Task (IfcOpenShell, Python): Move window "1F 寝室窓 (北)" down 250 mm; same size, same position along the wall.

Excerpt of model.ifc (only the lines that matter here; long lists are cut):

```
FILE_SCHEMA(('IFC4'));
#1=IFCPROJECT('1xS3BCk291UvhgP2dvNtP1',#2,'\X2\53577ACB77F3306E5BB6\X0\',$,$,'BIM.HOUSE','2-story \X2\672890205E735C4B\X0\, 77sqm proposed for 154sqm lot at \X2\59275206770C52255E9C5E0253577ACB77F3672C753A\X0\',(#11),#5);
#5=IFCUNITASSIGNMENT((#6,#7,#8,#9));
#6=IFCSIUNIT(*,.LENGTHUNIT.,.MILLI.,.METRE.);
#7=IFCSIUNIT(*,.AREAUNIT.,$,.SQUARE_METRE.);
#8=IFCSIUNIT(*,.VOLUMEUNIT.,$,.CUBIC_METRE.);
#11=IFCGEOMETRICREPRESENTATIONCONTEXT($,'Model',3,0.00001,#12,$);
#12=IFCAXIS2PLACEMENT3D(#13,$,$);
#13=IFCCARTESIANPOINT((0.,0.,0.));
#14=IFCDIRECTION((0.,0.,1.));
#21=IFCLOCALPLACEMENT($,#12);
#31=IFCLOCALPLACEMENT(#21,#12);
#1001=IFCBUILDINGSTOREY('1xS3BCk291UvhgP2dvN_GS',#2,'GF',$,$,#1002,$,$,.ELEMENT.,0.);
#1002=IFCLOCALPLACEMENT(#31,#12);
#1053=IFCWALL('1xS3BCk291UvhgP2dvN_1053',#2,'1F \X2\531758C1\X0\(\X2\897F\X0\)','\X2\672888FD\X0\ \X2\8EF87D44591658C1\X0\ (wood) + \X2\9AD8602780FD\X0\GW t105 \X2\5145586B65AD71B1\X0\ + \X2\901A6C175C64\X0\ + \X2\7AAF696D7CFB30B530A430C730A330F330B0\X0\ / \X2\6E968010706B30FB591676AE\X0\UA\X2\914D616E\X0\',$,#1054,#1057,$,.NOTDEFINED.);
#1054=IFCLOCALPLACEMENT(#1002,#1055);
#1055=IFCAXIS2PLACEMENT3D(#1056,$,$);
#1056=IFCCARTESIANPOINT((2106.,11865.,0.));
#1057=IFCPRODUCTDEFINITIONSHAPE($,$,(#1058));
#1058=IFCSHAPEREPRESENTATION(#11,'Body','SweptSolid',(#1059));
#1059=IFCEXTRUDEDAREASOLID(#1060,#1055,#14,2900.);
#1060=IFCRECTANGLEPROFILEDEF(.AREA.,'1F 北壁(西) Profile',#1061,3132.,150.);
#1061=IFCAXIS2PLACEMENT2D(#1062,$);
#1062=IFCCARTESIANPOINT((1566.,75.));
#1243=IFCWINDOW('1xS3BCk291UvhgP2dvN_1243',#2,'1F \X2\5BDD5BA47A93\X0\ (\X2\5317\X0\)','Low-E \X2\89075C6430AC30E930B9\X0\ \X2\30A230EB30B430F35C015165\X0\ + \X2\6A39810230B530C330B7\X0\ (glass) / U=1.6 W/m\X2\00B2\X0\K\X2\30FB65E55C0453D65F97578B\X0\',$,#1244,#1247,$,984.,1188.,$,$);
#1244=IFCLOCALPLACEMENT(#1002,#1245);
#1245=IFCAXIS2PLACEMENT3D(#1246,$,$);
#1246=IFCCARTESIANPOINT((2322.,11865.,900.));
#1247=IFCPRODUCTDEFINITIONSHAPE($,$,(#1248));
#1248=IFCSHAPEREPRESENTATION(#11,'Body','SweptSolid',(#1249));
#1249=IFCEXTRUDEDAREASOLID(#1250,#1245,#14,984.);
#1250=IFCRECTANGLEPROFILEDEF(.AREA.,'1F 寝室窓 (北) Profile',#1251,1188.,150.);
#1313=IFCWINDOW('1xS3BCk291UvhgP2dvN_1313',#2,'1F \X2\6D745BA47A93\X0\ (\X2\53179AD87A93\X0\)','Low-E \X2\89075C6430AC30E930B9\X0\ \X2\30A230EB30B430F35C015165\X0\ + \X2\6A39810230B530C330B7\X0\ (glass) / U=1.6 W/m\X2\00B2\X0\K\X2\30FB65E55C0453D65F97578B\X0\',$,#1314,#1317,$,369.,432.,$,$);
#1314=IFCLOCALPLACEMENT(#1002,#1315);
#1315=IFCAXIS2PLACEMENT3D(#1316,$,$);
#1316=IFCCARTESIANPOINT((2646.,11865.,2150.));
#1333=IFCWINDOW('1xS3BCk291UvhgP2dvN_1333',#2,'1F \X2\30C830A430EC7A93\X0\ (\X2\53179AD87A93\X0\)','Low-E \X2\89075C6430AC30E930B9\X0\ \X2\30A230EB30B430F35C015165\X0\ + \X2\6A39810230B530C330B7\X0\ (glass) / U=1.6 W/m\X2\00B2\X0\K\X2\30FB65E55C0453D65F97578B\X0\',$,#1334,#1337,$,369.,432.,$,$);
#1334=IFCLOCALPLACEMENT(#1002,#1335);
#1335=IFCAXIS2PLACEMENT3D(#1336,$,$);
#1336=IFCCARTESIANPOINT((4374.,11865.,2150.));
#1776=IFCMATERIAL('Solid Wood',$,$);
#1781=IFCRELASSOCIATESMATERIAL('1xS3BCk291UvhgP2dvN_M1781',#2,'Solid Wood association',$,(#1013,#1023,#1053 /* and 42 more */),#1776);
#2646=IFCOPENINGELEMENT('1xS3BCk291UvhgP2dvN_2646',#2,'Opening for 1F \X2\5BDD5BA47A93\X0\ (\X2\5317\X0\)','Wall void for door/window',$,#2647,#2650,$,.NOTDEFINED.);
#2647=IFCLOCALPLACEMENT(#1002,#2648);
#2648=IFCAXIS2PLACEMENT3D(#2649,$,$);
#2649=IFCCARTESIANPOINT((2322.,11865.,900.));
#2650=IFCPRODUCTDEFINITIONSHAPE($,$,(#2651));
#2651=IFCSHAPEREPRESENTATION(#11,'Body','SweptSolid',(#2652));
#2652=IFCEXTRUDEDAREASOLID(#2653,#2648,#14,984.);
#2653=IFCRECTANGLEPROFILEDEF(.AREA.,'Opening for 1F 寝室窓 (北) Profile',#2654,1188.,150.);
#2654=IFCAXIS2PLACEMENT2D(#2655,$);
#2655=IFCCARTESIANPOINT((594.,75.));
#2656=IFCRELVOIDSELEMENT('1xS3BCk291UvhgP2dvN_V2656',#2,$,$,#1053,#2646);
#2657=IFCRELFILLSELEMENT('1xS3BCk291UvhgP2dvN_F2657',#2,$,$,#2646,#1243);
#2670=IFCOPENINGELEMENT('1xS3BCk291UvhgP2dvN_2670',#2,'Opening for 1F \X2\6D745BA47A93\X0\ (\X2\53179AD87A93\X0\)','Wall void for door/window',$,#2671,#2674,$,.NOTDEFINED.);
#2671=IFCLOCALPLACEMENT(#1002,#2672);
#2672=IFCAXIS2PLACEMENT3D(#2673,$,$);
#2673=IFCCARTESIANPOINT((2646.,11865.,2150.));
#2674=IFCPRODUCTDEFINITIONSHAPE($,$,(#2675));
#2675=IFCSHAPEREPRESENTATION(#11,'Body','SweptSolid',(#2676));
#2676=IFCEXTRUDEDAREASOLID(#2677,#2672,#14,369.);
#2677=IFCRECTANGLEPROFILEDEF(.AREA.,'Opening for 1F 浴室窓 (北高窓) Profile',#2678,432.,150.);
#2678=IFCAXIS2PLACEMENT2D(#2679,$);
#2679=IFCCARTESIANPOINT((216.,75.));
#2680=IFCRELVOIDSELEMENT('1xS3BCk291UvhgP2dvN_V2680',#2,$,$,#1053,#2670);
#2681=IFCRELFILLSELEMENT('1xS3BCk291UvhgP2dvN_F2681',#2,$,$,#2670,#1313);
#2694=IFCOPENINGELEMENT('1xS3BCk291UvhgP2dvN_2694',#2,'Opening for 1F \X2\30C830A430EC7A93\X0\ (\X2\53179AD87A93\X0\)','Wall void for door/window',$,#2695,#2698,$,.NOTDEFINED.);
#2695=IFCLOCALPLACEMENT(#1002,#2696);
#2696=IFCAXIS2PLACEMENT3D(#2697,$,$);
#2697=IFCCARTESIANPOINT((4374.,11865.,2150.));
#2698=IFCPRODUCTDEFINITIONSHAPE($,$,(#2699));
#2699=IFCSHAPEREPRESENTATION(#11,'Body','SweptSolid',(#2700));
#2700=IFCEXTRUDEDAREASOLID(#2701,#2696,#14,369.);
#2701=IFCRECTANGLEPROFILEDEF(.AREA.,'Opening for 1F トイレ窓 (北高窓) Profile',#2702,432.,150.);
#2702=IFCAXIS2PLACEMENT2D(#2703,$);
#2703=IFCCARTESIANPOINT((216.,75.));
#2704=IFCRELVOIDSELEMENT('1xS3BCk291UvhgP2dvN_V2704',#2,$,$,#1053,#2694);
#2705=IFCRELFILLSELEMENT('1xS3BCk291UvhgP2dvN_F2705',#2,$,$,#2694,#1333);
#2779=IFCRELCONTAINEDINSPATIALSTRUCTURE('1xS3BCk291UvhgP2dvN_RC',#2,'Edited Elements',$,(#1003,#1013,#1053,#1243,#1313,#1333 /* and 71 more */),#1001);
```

```python
import numpy as np
import ifcopenshell
import ifcopenshell.api.geometry
import ifcopenshell.util.placement
import ifcopenshell.util.unit

model = ifcopenshell.open("model.ifc")
unit_scale = ifcopenshell.util.unit.calculate_unit_scale(model)

window = model.by_guid("1xS3BCk291UvhgP2dvN_1243")
opening = window.FillsVoids[0].RelatingOpeningElement
dz = -0.25 / unit_scale

shift = np.array([0.0, 0.0, dz])
# The window is not placed relative to its opening, so move both.
for product in (opening, window):
    matrix = ifcopenshell.util.placement.get_local_placement(product.ObjectPlacement)
    matrix[:3, 3] += shift
    ifcopenshell.api.geometry.edit_object_placement(model, product=product, matrix=matrix, is_si=False)

print(f"moved by {dz * unit_scale:+.3f} m")

model.write("model_edited.ifc")
```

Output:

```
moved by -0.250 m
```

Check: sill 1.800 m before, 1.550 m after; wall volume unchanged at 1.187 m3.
